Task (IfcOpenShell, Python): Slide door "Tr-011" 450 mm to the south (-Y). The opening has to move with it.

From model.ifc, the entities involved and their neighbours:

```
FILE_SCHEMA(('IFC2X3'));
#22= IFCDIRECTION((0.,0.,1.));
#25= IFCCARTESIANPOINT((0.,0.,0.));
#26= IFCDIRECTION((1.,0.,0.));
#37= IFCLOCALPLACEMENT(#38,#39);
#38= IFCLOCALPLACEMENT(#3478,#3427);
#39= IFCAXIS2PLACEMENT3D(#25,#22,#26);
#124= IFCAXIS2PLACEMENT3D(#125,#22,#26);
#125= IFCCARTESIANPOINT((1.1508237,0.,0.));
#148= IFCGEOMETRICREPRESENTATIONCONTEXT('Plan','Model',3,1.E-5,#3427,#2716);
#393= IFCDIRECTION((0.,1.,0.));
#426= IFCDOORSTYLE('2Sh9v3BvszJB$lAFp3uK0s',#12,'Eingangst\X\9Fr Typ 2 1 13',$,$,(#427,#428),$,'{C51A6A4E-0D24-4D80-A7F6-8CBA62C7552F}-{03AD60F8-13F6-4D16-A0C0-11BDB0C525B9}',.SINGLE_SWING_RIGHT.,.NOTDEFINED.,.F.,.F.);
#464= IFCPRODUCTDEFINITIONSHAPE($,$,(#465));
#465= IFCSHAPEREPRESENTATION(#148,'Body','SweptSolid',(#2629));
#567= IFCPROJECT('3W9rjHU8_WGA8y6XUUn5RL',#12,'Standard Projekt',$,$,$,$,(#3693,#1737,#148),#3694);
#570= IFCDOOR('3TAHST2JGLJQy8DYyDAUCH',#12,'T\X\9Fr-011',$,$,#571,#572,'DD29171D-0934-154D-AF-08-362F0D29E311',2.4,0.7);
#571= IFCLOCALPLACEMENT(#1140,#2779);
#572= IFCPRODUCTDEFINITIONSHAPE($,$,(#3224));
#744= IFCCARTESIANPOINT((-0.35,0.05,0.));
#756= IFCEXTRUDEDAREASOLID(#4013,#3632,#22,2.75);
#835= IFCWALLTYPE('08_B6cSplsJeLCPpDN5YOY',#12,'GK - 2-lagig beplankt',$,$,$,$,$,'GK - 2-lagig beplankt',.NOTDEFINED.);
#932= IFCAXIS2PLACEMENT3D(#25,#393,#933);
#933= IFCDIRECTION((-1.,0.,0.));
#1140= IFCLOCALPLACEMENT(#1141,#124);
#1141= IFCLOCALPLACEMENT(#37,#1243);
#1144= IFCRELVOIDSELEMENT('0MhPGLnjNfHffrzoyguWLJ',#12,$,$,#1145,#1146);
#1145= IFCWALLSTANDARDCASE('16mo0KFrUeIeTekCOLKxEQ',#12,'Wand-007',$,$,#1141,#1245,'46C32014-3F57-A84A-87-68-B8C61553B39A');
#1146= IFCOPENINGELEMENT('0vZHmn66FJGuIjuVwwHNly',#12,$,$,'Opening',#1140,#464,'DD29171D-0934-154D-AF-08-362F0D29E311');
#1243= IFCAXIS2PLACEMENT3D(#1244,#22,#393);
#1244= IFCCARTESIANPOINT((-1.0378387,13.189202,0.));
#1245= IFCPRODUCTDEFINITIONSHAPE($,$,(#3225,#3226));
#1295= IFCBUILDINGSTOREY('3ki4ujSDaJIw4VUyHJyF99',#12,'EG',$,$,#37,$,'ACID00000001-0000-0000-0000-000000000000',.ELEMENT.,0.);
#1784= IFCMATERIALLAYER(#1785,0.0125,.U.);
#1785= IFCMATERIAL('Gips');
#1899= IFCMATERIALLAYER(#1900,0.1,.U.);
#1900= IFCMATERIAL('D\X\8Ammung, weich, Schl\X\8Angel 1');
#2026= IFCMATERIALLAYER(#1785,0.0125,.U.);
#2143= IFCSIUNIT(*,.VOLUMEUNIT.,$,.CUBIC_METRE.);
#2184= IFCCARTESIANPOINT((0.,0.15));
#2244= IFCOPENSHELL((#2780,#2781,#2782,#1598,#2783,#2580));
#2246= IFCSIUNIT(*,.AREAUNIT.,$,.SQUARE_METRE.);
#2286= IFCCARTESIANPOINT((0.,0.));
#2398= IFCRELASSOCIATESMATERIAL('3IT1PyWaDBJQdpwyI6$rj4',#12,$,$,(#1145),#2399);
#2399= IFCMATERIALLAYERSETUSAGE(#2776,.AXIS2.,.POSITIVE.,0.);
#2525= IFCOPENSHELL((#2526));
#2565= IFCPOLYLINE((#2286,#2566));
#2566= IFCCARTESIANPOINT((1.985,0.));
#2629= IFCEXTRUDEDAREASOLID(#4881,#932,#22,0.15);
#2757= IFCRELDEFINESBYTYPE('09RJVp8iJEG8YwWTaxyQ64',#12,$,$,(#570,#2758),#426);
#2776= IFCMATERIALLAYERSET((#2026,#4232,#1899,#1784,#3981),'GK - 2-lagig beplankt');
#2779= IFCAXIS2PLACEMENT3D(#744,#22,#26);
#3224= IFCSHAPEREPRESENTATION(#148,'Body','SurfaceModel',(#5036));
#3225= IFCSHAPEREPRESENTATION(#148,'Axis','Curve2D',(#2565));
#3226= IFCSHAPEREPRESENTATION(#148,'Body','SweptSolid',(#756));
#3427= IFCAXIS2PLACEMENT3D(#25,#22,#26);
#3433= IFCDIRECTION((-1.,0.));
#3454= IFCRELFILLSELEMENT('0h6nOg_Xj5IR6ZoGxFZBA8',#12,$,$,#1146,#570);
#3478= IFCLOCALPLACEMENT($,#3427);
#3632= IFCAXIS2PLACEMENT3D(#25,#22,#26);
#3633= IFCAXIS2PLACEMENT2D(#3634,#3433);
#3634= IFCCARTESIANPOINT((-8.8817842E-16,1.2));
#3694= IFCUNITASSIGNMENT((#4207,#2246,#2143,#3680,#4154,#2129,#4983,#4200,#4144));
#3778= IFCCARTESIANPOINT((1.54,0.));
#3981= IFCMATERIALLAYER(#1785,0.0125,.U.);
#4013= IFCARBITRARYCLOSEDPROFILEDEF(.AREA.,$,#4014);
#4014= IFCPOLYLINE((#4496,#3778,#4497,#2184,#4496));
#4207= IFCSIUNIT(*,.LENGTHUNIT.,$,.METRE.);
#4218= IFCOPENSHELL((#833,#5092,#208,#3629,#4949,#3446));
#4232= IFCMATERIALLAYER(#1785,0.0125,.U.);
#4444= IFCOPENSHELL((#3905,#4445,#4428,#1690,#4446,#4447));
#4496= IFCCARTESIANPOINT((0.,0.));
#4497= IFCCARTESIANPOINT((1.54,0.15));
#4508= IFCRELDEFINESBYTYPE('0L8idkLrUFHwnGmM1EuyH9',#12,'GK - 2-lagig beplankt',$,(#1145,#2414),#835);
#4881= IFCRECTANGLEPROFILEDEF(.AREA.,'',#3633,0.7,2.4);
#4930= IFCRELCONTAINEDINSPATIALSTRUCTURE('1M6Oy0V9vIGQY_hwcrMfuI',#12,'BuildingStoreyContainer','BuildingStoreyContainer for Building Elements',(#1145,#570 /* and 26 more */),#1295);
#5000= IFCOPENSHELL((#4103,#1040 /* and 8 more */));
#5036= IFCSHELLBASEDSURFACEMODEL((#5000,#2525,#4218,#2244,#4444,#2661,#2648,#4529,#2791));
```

```python
import ifcopenshell
import ifcopenshell.api.geometry
import ifcopenshell.util.placement
import ifcopenshell.util.unit

model = ifcopenshell.open("model.ifc")
unit_scale = ifcopenshell.util.unit.calculate_unit_scale(model)

door = model.by_guid("3TAHST2JGLJQy8DYyDAUCH")
opening = door.FillsVoids[0].RelatingOpeningElement
wall = opening.VoidsElements[0].RelatingBuildingElement

wall_matrix = ifcopenshell.util.placement.get_local_placement(wall.ObjectPlacement)
shift = wall_matrix[:3, 0] * -0.45 / unit_scale
before = ifcopenshell.util.placement.get_local_placement(door.ObjectPlacement)[:3, 3].copy()

# The door is placed relative to its opening, so it follows when the opening moves.
matrix = ifcopenshell.util.placement.get_local_placement(opening.ObjectPlacement)
matrix[:3, 3] += shift
ifcopenshell.api.geometry.edit_object_placement(
    model, product=opening, matrix=matrix, is_si=False, should_transform_children=True
)

after = ifcopenshell.util.placement.get_local_placement(door.ObjectPlacement)[:3, 3]
print("door moved by", (after - before).round(3) + 0.0)

model.write("model_rev.ifc")
```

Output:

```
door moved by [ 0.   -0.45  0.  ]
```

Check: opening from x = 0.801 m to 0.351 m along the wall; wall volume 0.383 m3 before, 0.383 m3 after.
